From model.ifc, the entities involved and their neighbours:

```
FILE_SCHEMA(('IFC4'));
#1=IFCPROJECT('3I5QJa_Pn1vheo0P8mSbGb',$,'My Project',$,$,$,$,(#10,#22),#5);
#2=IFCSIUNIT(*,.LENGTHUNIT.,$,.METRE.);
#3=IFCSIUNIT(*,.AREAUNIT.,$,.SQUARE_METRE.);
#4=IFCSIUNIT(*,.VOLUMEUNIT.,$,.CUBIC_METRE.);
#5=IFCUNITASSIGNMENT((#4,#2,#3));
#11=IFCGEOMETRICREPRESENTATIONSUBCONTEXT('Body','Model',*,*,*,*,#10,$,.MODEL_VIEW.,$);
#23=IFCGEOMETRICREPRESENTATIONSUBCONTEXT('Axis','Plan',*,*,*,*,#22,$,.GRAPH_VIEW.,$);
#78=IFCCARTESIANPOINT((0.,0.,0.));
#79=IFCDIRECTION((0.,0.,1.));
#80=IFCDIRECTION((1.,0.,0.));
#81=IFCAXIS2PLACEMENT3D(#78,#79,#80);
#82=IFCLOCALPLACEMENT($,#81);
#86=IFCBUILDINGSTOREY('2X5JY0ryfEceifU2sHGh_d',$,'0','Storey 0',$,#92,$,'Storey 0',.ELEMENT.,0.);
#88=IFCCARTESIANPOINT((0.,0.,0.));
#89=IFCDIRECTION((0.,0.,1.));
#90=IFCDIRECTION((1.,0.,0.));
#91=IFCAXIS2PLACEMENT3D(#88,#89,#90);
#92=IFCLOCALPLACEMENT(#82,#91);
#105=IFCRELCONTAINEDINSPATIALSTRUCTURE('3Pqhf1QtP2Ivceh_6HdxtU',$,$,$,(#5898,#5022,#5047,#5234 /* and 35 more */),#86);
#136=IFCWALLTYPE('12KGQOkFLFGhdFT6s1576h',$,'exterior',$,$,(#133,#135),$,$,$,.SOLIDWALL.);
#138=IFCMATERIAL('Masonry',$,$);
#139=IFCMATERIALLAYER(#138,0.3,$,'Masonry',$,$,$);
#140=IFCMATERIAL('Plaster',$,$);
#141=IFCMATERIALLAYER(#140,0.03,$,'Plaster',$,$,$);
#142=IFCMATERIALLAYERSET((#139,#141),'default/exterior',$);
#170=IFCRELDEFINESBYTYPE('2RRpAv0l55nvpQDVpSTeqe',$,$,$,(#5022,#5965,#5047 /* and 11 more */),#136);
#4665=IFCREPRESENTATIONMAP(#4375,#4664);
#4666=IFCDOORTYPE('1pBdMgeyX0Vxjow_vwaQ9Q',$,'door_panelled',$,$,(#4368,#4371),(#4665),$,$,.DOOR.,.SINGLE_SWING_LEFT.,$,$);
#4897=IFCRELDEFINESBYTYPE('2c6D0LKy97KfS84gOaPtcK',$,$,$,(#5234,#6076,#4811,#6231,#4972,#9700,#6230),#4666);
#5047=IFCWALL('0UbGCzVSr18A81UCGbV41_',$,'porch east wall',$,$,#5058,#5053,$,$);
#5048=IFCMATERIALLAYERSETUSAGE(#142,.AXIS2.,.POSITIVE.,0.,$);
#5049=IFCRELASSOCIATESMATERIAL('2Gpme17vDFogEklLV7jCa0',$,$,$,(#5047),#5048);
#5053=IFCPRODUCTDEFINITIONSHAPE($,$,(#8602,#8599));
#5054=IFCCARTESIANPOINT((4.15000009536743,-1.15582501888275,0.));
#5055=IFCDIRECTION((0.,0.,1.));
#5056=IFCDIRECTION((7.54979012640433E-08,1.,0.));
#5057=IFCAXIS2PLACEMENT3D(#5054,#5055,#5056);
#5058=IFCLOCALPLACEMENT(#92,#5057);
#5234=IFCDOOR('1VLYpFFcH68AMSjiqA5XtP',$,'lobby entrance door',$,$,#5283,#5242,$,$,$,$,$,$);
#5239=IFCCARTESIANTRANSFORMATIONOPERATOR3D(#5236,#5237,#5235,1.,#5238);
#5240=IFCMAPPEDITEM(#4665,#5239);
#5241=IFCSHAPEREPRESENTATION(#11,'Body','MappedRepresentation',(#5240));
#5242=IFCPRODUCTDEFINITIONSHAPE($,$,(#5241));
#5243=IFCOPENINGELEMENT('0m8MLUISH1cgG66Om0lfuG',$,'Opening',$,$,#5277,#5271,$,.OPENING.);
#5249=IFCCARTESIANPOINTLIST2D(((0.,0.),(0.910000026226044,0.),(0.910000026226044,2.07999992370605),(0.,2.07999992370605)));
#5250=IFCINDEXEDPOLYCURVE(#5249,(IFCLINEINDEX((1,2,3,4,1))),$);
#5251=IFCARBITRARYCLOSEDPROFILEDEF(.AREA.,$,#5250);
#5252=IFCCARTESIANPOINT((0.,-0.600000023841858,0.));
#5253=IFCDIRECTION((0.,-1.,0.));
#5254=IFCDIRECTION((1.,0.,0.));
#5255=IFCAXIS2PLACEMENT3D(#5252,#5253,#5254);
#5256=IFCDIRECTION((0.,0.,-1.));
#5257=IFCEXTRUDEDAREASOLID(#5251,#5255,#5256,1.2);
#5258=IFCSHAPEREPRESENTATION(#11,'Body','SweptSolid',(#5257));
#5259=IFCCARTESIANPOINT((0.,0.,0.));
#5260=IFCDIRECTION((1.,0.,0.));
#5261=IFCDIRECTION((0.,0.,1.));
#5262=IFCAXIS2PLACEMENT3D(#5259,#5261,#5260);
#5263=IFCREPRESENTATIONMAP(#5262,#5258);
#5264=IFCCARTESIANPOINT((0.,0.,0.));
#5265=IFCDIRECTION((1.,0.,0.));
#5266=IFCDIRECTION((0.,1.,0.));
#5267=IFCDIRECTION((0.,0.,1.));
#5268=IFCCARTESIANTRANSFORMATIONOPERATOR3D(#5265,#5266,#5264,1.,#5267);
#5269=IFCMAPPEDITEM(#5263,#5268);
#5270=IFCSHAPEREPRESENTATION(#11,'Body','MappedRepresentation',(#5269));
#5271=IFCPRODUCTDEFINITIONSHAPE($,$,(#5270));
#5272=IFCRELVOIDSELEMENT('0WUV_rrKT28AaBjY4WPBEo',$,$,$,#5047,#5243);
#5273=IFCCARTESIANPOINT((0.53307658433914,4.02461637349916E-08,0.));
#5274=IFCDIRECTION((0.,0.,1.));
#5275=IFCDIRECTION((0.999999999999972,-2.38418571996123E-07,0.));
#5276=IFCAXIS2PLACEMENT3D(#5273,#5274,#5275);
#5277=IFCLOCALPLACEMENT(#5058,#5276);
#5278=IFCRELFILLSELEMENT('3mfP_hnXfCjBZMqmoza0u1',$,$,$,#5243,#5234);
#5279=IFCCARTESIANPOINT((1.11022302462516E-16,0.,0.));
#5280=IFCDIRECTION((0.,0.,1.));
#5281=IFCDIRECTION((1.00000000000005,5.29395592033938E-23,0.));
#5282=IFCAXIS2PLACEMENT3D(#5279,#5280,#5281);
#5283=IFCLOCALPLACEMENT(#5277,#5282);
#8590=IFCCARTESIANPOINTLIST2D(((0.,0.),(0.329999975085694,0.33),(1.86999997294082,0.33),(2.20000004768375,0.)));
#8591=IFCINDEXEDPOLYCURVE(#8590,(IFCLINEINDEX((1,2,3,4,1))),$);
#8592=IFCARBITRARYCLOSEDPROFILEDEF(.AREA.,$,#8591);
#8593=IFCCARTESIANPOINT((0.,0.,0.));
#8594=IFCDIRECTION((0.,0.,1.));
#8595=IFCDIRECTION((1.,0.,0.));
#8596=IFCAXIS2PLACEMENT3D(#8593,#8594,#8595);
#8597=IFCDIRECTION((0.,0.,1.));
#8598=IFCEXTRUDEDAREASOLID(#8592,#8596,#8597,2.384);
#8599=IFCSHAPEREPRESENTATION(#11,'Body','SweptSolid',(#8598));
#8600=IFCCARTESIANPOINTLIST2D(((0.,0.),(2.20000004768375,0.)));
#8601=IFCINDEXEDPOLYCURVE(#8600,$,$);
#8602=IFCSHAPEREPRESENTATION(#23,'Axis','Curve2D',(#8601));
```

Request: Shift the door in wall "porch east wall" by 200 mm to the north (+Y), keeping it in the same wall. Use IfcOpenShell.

```python
import ifcopenshell
import ifcopenshell.api.geometry
import ifcopenshell.util.placement

model = ifcopenshell.open("model.ifc")

door = model.by_guid("1VLYpFFcH68AMSjiqA5XtP")
opening = door.FillsVoids[0].RelatingOpeningElement
wall = opening.VoidsElements[0].RelatingBuildingElement

wall_matrix = ifcopenshell.util.placement.get_local_placement(wall.ObjectPlacement)
shift = wall_matrix[:3, 0] * 0.2
before = ifcopenshell.util.placement.get_local_placement(door.ObjectPlacement)[:3, 3].copy()

# The door is placed relative to its opening, so it follows when the opening moves.
matrix = ifcopenshell.util.placement.get_local_placement(opening.ObjectPlacement)
matrix[:3, 3] += shift
ifcopenshell.api.geometry.edit_object_placement(
    model, product=opening, matrix=matrix, is_si=False, should_transform_children=True
)

after = ifcopenshell.util.placement.get_local_placement(door.ObjectPlacement)[:3, 3]
print("door moved by", (after - before).round(3) + 0.0)

model.write("model-out.ifc")
```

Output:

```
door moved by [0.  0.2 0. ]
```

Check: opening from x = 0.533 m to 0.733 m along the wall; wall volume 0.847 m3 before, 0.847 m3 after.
